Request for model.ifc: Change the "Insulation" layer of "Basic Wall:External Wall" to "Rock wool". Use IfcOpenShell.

First a look at what the model holds.

```python
import ifcopenshell
import ifcopenshell.util.element

model = ifcopenshell.open("model.ifc")
print(model.schema)
for layer_set in model.by_type("IfcMaterialLayerSet"):
    if layer_set.LayerSetName == "Basic Wall:External Wall":
        for layer in layer_set.MaterialLayers:
            print(layer.id(), layer.Material and layer.Material.Name, layer.LayerThickness, sep=" | ")
        print(len(ifcopenshell.util.element.get_elements_by_material(model, layer_set)), "elements and types use it")
print(sorted(m.Name for m in model.by_type("IfcMaterial") if m.Name)[:60])
```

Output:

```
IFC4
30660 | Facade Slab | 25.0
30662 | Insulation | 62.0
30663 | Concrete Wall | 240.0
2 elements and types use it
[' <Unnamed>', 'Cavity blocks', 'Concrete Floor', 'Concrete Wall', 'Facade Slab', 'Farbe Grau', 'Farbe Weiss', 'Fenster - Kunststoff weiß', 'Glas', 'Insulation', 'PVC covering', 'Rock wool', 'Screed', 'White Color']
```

```python
import ifcopenshell
import ifcopenshell.api.material

model = ifcopenshell.open("model.ifc")

layer_set = next(s for s in model.by_type("IfcMaterialLayerSet") if s.LayerSetName == "Basic Wall:External Wall")
layer = next(l for l in layer_set.MaterialLayers if l.Material and l.Material.Name == "Insulation")
material = next(m for m in model.by_type("IfcMaterial") if m.Name == "Rock wool")

# Point this one layer at the other material; renaming the old one would change it everywhere.
ifcopenshell.api.material.edit_layer(model, layer=layer, attributes={}, material=material)

print([l.Material.Name if l.Material else None for l in layer_set.MaterialLayers])

model.write("model-out.ifc")
```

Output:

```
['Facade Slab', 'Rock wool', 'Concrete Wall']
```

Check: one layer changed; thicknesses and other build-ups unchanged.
